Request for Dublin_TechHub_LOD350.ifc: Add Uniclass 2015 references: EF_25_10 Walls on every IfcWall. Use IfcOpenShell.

First a look at what the model holds.

```python
import ifcopenshell

model = ifcopenshell.open("Dublin_TechHub_LOD350.ifc")
print(model.schema)
print("classifications:", [c.Name for c in model.by_type("IfcClassification")])
for ifc_class in ("IfcDoor", "IfcRoof", "IfcStair", "IfcWall", "IfcWindow"):
    print(ifc_class, len(model.by_type(ifc_class)))
```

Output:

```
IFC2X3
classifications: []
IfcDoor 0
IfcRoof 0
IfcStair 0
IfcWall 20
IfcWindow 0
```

```python
import ifcopenshell
import ifcopenshell.api.classification

model = ifcopenshell.open("Dublin_TechHub_LOD350.ifc")

# IFC2X3 requires Source and Edition and has no link from the project to the system.
system = model.create_entity("IfcClassification", Source="NBS", Edition="2015", Name="Uniclass 2015")

codes = {
    "IfcWall": ("EF_25_10", "Walls"),
}
for ifc_class, (code, name) in codes.items():
    products = model.by_type(ifc_class)
    ifcopenshell.api.classification.add_reference(
        model, products=products, classification=system, identification=code, name=name
    )
    print(code, len(products))

model.write("Dublin_TechHub_LOD350_v2.ifc")
```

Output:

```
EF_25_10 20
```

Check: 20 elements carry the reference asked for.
